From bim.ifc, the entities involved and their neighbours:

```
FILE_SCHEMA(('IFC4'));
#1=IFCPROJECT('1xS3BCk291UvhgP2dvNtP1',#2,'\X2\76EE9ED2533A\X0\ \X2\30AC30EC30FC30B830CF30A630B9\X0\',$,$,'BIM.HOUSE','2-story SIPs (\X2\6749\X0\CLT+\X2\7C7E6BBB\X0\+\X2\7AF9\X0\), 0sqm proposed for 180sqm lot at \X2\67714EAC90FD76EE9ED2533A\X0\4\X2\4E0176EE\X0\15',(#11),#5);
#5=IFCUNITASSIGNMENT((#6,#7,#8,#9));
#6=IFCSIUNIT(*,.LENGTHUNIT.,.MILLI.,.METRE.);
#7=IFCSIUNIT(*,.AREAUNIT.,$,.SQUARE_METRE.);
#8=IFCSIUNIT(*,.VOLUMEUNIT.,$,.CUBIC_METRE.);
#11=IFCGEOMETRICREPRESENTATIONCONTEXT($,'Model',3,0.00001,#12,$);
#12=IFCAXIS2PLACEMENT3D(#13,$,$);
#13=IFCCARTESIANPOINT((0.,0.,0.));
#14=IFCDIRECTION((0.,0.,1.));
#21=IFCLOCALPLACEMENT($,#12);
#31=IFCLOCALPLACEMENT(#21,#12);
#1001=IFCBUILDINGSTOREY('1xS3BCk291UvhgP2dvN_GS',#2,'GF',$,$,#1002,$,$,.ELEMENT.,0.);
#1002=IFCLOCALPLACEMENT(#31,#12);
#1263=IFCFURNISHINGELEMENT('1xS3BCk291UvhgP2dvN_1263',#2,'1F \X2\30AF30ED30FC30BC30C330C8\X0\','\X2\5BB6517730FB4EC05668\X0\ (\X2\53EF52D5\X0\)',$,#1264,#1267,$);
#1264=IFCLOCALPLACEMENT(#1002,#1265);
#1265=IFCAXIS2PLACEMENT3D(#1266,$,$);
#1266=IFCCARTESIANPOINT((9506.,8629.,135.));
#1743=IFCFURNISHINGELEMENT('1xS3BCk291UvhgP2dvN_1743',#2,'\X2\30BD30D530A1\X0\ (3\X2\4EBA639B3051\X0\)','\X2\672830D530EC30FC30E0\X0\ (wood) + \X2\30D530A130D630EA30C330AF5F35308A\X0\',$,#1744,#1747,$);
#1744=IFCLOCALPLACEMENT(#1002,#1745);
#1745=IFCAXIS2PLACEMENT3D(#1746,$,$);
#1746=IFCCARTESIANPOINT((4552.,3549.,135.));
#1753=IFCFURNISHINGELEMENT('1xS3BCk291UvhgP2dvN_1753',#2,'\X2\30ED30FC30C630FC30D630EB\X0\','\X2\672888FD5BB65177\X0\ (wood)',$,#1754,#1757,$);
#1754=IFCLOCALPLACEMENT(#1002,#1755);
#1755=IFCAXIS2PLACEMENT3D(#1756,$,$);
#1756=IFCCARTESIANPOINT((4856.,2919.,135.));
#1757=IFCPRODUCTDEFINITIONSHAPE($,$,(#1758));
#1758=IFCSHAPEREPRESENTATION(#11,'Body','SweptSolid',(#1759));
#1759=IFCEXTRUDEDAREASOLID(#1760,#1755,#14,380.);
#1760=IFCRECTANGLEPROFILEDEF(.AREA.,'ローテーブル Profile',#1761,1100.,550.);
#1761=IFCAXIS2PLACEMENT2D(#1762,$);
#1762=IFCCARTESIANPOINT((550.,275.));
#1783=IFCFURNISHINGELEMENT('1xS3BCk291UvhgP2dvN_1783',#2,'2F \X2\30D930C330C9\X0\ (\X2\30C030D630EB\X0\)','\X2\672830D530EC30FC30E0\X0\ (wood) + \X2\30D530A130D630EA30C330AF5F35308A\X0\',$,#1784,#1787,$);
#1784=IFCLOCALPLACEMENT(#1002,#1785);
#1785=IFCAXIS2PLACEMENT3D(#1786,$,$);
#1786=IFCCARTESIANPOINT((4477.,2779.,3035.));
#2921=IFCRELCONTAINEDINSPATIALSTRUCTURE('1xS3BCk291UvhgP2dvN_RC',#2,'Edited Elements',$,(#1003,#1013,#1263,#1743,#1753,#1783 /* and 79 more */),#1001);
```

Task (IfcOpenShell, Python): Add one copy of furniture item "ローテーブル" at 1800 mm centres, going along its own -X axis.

```python
import ifcopenshell
import ifcopenshell.api.geometry
import ifcopenshell.api.root
import ifcopenshell.util.element
import ifcopenshell.util.placement
import ifcopenshell.util.unit

model = ifcopenshell.open("bim.ifc")
unit_scale = ifcopenshell.util.unit.calculate_unit_scale(model)


def reuse_history(source, copy):
    """copy_class also copies each property set's owner history, people and application; keep the originals."""
    for rel in copy.IsDefinedBy:
        if rel.is_a("IfcRelDefinesByProperties") and (history := rel.RelatingPropertyDefinition.OwnerHistory):
            rel.RelatingPropertyDefinition.OwnerHistory = source.OwnerHistory
            ifcopenshell.util.element.remove_deep2(model, history)


source = model.by_guid("1xS3BCk291UvhgP2dvN_1753")
base = ifcopenshell.util.placement.get_local_placement(source.ObjectPlacement)
step = -base[:3, 0] * 1.8 / unit_scale

for i in range(1, 2):
    copy = ifcopenshell.api.root.copy_class(model, product=source)
    copy.Representation = ifcopenshell.util.element.copy_deep(
        model, source.Representation, exclude=["IfcGeometricRepresentationContext", "IfcRepresentationMap"]
    )
    reuse_history(source, copy)
    matrix = base.copy()
    matrix[:3, 3] += i * step
    print("added at", matrix[:3, 3].round(3) + 0.0)
    ifcopenshell.api.geometry.edit_object_placement(model, product=copy, matrix=matrix, is_si=False)

model.write("bim_v2.ifc")
```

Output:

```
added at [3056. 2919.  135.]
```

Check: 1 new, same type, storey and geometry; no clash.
